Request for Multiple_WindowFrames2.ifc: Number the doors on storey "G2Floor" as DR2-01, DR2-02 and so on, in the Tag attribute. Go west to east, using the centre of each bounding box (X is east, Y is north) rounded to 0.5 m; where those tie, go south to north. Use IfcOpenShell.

First a look at what the model holds.

```python
import ifcopenshell
import ifcopenshell.util.element
import ifcopenshell.util.placement

model = ifcopenshell.open("Multiple_WindowFrames2.ifc")
print(model.schema)
storey = next(s for s in model.by_type("IfcBuildingStorey") if s.Name == "G2Floor")
doors = [e for e in ifcopenshell.util.element.get_decomposition(storey) if e.is_a("IfcDoor")]
for e in sorted(doors, key=lambda e: e.id()):
    origin = ifcopenshell.util.placement.get_local_placement(e.ObjectPlacement)[:3, 3]
    print(e.id(), e.Tag, e.Name, origin.round(2) + 0.0, sep=" | ")
```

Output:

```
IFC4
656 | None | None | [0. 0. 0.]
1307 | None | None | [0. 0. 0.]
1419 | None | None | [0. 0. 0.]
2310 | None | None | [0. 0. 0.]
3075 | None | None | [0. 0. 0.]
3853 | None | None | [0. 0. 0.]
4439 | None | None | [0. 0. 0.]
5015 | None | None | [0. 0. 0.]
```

```python
import ifcopenshell
import ifcopenshell.geom
import ifcopenshell.util.element
import ifcopenshell.util.shape

model = ifcopenshell.open("Multiple_WindowFrames2.ifc")
settings = ifcopenshell.geom.settings()
settings.set("use-world-coords", True)


def centre(element):
    shape = ifcopenshell.geom.create_shape(settings, element)
    return ifcopenshell.util.shape.get_bbox_centroid(shape.geometry)


storey = next(s for s in model.by_type("IfcBuildingStorey") if s.Name == "G2Floor")
doors = [e for e in ifcopenshell.util.element.get_decomposition(storey) if e.is_a("IfcDoor")]

# Insertion points can sit at a corner or the storey origin, so sort by the geometry (in metres).
centres = {e: centre(e) for e in doors}
doors.sort(key=lambda e: (round(centres[e][0] / 0.5), centres[e][1]))

for i, e in enumerate(doors, start=1):
    number = f"DR2-{i:02d}"
    e.Tag = number
    print(e.id(), number)

model.write("Multiple_WindowFrames2_v2.ifc")
```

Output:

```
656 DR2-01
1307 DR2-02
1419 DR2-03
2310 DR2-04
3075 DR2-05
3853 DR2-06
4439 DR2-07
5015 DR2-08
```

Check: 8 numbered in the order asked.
